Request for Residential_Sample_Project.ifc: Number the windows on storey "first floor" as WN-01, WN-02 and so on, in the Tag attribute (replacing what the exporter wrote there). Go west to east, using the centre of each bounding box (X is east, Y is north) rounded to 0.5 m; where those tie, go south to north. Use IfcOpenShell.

First a look at what the model holds.

```python
import ifcopenshell
import ifcopenshell.util.element
import ifcopenshell.util.placement

model = ifcopenshell.open("Residential_Sample_Project.ifc")
print(model.schema)
storey = next(s for s in model.by_type("IfcBuildingStorey") if s.Name == "first floor")
windows = [e for e in ifcopenshell.util.element.get_decomposition(storey) if e.is_a("IfcWindow")]
for e in sorted(windows, key=lambda e: e.id()):
    origin = ifcopenshell.util.placement.get_local_placement(e.ObjectPlacement)[:3, 3]
    print(e.id(), e.Tag, e.Name, origin.round(2) + 0.0, sep=" | ")
```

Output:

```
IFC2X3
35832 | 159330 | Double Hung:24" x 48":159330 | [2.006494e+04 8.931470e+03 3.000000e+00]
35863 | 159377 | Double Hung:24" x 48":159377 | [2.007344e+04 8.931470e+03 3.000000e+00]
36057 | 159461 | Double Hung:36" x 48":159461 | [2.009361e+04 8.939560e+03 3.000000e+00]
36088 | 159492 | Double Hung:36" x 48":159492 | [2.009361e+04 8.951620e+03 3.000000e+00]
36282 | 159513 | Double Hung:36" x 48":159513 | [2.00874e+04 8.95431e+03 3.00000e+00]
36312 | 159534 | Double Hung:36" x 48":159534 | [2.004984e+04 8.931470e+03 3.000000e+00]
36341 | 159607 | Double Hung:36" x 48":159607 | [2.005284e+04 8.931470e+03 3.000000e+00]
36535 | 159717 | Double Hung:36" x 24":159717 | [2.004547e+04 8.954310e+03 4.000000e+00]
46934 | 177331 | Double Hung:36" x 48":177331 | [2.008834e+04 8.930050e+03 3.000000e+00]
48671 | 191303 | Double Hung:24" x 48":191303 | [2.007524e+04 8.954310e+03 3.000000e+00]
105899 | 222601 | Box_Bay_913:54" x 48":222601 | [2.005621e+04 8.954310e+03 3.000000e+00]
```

```python
import ifcopenshell
import ifcopenshell.geom
import ifcopenshell.util.element
import ifcopenshell.util.shape

model = ifcopenshell.open("Residential_Sample_Project.ifc")
settings = ifcopenshell.geom.settings()
settings.set("use-world-coords", True)


def centre(element):
    shape = ifcopenshell.geom.create_shape(settings, element)
    return ifcopenshell.util.shape.get_bbox_centroid(shape.geometry)


storey = next(s for s in model.by_type("IfcBuildingStorey") if s.Name == "first floor")
windows = [e for e in ifcopenshell.util.element.get_decomposition(storey) if e.is_a("IfcWindow")]

# Insertion points can sit at a corner or the storey origin, so sort by the geometry (in metres).
centres = {e: centre(e) for e in windows}
windows.sort(key=lambda e: (round(centres[e][0] / 0.5), centres[e][1]))

for i, e in enumerate(windows, start=1):
    number = f"WN-{i:02d}"
    e.Tag = number
    print(e.id(), number)

model.write("Residential_Sample_Project_v2.ifc")
```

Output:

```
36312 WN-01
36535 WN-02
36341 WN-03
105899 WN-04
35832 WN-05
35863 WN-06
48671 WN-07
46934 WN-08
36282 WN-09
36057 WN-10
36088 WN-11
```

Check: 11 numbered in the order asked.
